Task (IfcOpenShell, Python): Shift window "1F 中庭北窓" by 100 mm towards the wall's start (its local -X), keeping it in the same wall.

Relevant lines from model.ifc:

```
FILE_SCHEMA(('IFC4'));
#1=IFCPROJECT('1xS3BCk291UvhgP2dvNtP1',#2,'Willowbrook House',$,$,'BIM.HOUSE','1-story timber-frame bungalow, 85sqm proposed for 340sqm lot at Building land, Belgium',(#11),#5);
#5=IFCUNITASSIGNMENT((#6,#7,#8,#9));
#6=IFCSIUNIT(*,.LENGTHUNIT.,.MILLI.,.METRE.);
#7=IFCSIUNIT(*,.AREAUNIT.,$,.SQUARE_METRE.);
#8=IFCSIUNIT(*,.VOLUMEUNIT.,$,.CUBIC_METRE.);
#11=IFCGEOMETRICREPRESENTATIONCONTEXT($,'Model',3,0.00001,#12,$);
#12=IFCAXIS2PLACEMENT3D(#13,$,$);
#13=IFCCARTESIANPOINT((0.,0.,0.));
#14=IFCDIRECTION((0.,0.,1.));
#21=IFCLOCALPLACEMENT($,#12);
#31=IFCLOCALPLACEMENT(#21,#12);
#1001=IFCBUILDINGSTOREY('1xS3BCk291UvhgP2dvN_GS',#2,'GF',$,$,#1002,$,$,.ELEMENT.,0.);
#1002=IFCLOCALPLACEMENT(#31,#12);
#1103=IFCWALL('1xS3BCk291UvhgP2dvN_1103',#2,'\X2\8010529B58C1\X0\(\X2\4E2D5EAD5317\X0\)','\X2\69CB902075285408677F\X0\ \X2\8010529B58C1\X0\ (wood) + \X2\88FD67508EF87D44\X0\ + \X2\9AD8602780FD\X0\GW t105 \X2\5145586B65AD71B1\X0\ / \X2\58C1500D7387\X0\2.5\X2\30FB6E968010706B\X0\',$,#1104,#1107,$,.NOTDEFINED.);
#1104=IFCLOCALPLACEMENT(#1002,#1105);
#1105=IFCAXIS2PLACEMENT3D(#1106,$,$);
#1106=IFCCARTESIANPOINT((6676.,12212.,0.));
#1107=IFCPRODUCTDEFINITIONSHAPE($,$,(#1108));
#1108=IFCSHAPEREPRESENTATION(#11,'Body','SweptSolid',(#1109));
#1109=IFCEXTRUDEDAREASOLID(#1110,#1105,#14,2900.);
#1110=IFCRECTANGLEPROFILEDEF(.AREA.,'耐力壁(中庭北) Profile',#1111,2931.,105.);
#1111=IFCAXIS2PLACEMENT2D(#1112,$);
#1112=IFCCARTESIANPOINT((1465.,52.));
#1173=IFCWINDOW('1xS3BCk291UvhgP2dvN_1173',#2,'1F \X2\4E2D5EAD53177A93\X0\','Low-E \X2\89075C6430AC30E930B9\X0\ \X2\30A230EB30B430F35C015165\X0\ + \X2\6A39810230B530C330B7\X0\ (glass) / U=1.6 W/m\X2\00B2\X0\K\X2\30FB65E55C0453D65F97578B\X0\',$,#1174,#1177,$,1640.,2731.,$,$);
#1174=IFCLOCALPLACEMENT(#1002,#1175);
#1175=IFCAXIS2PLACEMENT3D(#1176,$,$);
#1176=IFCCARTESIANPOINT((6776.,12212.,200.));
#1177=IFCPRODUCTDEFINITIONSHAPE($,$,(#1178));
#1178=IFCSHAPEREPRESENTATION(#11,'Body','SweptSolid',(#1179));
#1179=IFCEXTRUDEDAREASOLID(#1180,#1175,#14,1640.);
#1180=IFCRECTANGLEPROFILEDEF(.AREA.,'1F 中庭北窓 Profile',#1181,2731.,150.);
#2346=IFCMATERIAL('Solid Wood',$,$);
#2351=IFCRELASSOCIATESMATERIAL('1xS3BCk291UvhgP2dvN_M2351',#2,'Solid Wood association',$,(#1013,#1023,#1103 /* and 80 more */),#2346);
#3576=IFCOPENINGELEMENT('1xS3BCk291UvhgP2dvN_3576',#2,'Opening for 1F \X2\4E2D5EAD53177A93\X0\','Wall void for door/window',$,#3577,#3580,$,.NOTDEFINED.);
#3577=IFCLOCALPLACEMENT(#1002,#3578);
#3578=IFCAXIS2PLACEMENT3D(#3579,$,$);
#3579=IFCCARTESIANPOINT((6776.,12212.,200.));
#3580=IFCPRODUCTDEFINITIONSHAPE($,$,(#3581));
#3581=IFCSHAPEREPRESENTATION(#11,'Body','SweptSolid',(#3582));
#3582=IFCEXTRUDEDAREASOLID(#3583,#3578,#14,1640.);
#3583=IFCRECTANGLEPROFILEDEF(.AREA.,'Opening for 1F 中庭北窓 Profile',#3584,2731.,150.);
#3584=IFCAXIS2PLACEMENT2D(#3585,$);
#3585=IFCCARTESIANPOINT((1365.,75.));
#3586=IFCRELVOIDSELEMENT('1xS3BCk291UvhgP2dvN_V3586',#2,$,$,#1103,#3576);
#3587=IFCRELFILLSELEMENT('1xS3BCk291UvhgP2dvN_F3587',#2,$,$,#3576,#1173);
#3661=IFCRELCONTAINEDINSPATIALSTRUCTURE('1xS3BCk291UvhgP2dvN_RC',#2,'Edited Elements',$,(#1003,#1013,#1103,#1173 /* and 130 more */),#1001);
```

```python
import ifcopenshell
import ifcopenshell.api.geometry
import ifcopenshell.util.placement
import ifcopenshell.util.unit

model = ifcopenshell.open("model.ifc")
unit_scale = ifcopenshell.util.unit.calculate_unit_scale(model)

window = model.by_guid("1xS3BCk291UvhgP2dvN_1173")
opening = window.FillsVoids[0].RelatingOpeningElement
wall = opening.VoidsElements[0].RelatingBuildingElement

wall_matrix = ifcopenshell.util.placement.get_local_placement(wall.ObjectPlacement)
shift = wall_matrix[:3, 0] * -0.1 / unit_scale
before = ifcopenshell.util.placement.get_local_placement(window.ObjectPlacement)[:3, 3].copy()

# The window is not placed relative to its opening, so move both.
for product in (opening, window):
    matrix = ifcopenshell.util.placement.get_local_placement(product.ObjectPlacement)
    matrix[:3, 3] += shift
    ifcopenshell.api.geometry.edit_object_placement(model, product=product, matrix=matrix, is_si=False)

after = ifcopenshell.util.placement.get_local_placement(window.ObjectPlacement)[:3, 3]
print("window moved by", (after - before).round(3) + 0.0)

model.write("model_rev.ifc")
```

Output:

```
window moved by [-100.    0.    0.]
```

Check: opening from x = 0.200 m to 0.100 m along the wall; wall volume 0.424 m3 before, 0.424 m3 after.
